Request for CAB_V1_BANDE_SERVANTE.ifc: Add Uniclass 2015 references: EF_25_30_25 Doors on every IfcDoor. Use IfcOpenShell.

First a look at what the model holds.

```python
import ifcopenshell

model = ifcopenshell.open("CAB_V1_BANDE_SERVANTE.ifc")
print(model.schema)
print("classifications:", [c.Name for c in model.by_type("IfcClassification")])
for ifc_class in ("IfcDoor", "IfcRoof", "IfcStair", "IfcWall", "IfcWindow"):
    print(ifc_class, len(model.by_type(ifc_class)))
```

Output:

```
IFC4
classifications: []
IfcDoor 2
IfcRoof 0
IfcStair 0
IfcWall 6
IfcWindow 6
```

```python
import ifcopenshell
import ifcopenshell.api.classification

model = ifcopenshell.open("CAB_V1_BANDE_SERVANTE.ifc")

system = ifcopenshell.api.classification.add_classification(model, classification="Uniclass 2015")

codes = {
    "IfcDoor": ("EF_25_30_25", "Doors"),
}
for ifc_class, (code, name) in codes.items():
    products = model.by_type(ifc_class)
    ifcopenshell.api.classification.add_reference(
        model, products=products, classification=system, identification=code, name=name
    )
    print(code, len(products))

model.write("CAB_V1_BANDE_SERVANTE_updated.ifc")
```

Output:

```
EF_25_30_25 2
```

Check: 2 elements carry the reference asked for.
